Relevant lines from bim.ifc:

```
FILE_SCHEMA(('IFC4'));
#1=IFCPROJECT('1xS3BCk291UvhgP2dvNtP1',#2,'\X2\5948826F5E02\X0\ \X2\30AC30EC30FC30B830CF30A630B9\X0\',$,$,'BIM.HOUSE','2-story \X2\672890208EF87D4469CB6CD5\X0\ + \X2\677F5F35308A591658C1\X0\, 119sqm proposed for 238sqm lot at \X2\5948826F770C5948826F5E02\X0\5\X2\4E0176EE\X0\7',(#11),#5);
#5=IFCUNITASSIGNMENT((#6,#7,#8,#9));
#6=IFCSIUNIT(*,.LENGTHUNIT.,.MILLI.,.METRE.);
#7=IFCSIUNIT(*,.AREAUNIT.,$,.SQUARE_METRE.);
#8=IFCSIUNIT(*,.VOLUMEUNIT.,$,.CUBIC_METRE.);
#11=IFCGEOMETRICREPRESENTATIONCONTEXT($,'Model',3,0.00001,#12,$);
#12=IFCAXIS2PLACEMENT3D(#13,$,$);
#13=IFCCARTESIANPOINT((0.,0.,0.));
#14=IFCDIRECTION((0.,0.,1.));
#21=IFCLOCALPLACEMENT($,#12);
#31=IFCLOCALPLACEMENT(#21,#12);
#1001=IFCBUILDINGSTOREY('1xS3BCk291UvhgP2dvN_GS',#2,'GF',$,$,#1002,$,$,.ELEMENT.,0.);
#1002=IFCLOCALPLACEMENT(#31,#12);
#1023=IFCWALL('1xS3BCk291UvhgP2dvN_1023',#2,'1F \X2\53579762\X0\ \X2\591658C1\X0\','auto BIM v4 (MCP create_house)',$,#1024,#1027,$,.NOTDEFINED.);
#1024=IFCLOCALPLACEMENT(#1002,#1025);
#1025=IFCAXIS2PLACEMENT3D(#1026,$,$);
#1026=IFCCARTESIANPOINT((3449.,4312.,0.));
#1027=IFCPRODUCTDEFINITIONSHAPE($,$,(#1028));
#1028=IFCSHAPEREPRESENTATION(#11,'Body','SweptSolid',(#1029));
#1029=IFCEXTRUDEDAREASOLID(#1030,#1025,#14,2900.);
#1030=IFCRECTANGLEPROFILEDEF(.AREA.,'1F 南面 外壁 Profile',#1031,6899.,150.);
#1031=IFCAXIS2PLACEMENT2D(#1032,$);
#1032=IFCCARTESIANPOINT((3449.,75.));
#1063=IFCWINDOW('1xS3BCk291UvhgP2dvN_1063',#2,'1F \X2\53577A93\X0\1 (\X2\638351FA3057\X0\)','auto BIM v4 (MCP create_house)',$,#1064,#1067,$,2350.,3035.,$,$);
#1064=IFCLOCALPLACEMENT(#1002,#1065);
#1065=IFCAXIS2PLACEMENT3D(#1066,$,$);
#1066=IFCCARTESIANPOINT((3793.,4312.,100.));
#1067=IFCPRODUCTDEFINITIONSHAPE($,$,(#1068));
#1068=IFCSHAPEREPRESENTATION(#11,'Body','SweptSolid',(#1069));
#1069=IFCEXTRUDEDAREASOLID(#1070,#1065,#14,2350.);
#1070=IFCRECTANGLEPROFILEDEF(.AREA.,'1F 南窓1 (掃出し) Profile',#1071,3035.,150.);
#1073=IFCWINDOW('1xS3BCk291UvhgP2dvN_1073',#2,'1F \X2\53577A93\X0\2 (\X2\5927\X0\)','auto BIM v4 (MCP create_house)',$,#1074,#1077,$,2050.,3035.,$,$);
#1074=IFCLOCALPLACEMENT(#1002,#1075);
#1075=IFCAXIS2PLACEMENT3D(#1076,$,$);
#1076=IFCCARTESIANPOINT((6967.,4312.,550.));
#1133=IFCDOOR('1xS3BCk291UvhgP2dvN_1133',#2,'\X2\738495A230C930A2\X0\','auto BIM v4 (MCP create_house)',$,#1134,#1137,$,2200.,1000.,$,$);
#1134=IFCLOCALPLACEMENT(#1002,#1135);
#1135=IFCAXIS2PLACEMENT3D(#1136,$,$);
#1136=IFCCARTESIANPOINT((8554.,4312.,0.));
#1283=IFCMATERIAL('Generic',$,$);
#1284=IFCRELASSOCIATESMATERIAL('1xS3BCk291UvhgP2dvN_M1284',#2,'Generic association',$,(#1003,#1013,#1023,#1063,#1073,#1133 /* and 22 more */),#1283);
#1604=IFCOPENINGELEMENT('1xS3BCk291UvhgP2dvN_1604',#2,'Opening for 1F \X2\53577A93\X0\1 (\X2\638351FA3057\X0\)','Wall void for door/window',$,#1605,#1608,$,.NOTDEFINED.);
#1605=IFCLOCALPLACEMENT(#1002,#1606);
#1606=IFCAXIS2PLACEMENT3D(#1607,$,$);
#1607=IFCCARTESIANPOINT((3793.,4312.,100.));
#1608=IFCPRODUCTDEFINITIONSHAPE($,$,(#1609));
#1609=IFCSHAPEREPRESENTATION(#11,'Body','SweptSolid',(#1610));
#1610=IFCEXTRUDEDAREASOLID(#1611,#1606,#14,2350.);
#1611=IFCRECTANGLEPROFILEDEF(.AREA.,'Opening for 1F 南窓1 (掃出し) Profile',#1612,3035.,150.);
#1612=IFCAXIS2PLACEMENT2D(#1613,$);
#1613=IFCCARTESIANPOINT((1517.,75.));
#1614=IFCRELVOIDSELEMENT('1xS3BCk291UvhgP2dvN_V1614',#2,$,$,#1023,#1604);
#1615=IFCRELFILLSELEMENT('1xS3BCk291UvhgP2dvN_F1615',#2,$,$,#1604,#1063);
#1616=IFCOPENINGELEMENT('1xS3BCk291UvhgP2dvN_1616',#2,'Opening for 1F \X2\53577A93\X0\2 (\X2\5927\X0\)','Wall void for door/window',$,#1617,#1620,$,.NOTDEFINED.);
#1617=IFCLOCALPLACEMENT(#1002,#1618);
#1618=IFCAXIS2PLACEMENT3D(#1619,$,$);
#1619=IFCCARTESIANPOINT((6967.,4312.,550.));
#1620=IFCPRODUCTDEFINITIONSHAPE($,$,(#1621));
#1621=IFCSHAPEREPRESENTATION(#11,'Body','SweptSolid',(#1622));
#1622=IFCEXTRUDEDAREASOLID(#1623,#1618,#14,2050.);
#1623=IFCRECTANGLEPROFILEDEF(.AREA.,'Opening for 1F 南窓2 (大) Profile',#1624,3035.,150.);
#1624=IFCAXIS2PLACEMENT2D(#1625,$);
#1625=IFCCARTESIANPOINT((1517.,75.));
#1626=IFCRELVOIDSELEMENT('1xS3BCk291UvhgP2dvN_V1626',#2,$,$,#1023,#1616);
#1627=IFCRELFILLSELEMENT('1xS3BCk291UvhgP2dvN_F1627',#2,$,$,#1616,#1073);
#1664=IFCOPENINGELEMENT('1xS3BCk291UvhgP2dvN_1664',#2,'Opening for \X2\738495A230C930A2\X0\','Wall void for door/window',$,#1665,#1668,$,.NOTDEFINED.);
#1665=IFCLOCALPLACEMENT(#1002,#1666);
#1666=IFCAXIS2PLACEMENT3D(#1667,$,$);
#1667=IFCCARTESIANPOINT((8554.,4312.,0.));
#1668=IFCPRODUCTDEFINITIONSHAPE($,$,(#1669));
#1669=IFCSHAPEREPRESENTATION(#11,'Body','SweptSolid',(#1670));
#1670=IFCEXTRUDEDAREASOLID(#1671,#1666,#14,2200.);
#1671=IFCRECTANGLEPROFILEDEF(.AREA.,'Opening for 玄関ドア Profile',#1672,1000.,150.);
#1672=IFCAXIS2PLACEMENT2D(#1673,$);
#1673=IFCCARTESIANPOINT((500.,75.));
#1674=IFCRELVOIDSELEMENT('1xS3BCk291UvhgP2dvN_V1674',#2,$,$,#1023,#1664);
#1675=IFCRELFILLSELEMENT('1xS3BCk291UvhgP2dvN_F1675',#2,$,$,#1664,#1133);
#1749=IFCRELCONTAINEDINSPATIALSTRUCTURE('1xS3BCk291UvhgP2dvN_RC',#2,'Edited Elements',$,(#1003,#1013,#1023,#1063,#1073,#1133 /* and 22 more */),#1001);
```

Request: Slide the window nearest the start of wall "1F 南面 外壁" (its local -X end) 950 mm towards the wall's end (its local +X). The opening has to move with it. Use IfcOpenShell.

```python
import ifcopenshell
import ifcopenshell.api.geometry
import ifcopenshell.util.placement
import ifcopenshell.util.unit

model = ifcopenshell.open("bim.ifc")
unit_scale = ifcopenshell.util.unit.calculate_unit_scale(model)

window = model.by_id(1063)
opening = window.FillsVoids[0].RelatingOpeningElement
wall = opening.VoidsElements[0].RelatingBuildingElement

wall_matrix = ifcopenshell.util.placement.get_local_placement(wall.ObjectPlacement)
shift = wall_matrix[:3, 0] * 0.95 / unit_scale
before = ifcopenshell.util.placement.get_local_placement(window.ObjectPlacement)[:3, 3].copy()

# The window is not placed relative to its opening, so move both.
for product in (opening, window):
    matrix = ifcopenshell.util.placement.get_local_placement(product.ObjectPlacement)
    matrix[:3, 3] += shift
    ifcopenshell.api.geometry.edit_object_placement(model, product=product, matrix=matrix, is_si=False)

after = ifcopenshell.util.placement.get_local_placement(window.ObjectPlacement)[:3, 3]
print("window moved by", (after - before).round(3) + 0.0)

model.write("bim_v2.ifc")
```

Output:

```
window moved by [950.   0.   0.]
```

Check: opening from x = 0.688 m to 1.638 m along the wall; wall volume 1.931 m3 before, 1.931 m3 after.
